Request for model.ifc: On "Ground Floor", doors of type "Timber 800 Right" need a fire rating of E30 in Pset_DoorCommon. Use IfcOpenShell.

First a look at what the model holds.

```python
import ifcopenshell
import ifcopenshell.util.element

model = ifcopenshell.open("model.ifc")
print(model.schema)
storey = next(s for s in model.by_type("IfcBuildingStorey") if s.Name == "Ground Floor")
doors = [e for e in ifcopenshell.util.element.get_decomposition(storey) if e.is_a("IfcDoor")]
seen = {}
for e in doors:
    element_type = ifcopenshell.util.element.get_type(e)
    key = (element_type.Name if element_type != e and element_type else None, ifcopenshell.util.element.get_pset(e, "Pset_DoorCommon", "FireRating"))
    seen[key] = seen.get(key, 0) + 1
for (name, value), count in sorted(seen.items(), key=str):
    print(count, "x", name, "|", value)
```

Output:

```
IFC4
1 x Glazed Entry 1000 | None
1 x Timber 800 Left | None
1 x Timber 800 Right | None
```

```python
import ifcopenshell
import ifcopenshell.api.pset
import ifcopenshell.util.element

model = ifcopenshell.open("model.ifc")

storey = next(s for s in model.by_type("IfcBuildingStorey") if s.Name == "Ground Floor")
doors = [e for e in ifcopenshell.util.element.get_decomposition(storey) if e.is_a("IfcDoor")]

count = 0
for e in doors:
    element_type = ifcopenshell.util.element.get_type(e)
    if element_type in (None, e) or element_type.Name != "Timber 800 Right":
        continue
    # add_pset returns the element's existing set when there is one.
    pset = ifcopenshell.api.pset.add_pset(model, product=e, name="Pset_DoorCommon")
    ifcopenshell.api.pset.edit_pset(model, pset=pset, properties={"FireRating": "E30"})
    count += 1

print(count, "doors updated")

model.write("model-out.ifc")
```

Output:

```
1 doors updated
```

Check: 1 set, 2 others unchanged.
